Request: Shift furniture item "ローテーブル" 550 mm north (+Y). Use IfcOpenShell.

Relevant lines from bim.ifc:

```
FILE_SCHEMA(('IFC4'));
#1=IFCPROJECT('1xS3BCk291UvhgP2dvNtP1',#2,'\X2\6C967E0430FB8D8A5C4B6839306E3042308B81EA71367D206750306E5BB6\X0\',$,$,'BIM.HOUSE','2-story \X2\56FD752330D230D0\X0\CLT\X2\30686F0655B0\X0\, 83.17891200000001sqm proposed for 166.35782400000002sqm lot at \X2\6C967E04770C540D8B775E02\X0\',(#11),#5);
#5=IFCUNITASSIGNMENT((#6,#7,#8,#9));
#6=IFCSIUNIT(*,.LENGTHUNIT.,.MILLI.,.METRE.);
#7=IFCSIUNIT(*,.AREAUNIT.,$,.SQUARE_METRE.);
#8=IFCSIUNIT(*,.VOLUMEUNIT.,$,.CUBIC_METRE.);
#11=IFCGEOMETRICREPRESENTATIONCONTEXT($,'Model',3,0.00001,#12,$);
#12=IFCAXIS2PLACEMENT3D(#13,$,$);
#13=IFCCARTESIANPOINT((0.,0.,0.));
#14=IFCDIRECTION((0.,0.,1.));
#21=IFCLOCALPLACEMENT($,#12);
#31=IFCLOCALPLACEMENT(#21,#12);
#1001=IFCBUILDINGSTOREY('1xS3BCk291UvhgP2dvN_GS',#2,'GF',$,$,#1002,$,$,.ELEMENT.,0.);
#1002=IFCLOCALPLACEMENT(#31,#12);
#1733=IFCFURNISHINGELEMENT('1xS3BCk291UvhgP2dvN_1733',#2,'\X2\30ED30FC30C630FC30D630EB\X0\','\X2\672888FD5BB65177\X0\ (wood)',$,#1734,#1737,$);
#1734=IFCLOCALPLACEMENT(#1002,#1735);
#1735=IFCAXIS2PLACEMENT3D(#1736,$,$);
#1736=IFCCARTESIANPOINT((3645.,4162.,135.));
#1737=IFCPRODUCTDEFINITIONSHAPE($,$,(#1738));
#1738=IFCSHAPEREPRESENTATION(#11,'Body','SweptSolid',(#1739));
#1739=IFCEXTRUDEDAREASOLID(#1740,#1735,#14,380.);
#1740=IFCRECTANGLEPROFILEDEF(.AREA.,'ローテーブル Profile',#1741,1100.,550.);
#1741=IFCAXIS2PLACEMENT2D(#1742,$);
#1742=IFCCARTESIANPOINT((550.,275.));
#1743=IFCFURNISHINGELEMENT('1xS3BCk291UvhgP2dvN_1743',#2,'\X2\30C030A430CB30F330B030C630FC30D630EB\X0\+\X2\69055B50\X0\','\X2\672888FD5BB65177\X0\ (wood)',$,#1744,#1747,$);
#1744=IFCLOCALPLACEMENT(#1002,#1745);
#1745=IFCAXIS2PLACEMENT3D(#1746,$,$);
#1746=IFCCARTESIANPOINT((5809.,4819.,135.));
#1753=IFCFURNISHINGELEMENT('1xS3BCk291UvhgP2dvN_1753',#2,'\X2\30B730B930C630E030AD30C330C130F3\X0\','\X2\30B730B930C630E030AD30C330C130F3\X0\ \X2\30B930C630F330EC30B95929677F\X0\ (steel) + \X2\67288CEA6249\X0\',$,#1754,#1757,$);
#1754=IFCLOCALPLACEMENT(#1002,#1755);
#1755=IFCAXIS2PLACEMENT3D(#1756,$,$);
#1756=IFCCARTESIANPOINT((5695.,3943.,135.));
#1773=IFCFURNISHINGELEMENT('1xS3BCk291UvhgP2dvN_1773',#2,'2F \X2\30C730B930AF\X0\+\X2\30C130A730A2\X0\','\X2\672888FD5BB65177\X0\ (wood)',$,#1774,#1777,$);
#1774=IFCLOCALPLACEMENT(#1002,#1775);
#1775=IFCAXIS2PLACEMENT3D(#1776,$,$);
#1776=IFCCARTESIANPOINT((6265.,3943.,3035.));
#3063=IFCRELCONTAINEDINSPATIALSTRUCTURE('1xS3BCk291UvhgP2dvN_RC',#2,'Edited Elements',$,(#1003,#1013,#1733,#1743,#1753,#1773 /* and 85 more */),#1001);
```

```python
import ifcopenshell
import ifcopenshell.api.geometry
import ifcopenshell.util.placement
import ifcopenshell.util.unit

model = ifcopenshell.open("bim.ifc")
unit_scale = ifcopenshell.util.unit.calculate_unit_scale(model)

item = model.by_id(1733)
matrix = ifcopenshell.util.placement.get_local_placement(item.ObjectPlacement)
matrix[1, 3] += 0.55 / unit_scale
ifcopenshell.api.geometry.edit_object_placement(model, product=item, matrix=matrix, is_si=False)

print(ifcopenshell.util.placement.get_local_placement(item.ObjectPlacement).round(3) + 0.0)

model.write("bim_updated.ifc")
```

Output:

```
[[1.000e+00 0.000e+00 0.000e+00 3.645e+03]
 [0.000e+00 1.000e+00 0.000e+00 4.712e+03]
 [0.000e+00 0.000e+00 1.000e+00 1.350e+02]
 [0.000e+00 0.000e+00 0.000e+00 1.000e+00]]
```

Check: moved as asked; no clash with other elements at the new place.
